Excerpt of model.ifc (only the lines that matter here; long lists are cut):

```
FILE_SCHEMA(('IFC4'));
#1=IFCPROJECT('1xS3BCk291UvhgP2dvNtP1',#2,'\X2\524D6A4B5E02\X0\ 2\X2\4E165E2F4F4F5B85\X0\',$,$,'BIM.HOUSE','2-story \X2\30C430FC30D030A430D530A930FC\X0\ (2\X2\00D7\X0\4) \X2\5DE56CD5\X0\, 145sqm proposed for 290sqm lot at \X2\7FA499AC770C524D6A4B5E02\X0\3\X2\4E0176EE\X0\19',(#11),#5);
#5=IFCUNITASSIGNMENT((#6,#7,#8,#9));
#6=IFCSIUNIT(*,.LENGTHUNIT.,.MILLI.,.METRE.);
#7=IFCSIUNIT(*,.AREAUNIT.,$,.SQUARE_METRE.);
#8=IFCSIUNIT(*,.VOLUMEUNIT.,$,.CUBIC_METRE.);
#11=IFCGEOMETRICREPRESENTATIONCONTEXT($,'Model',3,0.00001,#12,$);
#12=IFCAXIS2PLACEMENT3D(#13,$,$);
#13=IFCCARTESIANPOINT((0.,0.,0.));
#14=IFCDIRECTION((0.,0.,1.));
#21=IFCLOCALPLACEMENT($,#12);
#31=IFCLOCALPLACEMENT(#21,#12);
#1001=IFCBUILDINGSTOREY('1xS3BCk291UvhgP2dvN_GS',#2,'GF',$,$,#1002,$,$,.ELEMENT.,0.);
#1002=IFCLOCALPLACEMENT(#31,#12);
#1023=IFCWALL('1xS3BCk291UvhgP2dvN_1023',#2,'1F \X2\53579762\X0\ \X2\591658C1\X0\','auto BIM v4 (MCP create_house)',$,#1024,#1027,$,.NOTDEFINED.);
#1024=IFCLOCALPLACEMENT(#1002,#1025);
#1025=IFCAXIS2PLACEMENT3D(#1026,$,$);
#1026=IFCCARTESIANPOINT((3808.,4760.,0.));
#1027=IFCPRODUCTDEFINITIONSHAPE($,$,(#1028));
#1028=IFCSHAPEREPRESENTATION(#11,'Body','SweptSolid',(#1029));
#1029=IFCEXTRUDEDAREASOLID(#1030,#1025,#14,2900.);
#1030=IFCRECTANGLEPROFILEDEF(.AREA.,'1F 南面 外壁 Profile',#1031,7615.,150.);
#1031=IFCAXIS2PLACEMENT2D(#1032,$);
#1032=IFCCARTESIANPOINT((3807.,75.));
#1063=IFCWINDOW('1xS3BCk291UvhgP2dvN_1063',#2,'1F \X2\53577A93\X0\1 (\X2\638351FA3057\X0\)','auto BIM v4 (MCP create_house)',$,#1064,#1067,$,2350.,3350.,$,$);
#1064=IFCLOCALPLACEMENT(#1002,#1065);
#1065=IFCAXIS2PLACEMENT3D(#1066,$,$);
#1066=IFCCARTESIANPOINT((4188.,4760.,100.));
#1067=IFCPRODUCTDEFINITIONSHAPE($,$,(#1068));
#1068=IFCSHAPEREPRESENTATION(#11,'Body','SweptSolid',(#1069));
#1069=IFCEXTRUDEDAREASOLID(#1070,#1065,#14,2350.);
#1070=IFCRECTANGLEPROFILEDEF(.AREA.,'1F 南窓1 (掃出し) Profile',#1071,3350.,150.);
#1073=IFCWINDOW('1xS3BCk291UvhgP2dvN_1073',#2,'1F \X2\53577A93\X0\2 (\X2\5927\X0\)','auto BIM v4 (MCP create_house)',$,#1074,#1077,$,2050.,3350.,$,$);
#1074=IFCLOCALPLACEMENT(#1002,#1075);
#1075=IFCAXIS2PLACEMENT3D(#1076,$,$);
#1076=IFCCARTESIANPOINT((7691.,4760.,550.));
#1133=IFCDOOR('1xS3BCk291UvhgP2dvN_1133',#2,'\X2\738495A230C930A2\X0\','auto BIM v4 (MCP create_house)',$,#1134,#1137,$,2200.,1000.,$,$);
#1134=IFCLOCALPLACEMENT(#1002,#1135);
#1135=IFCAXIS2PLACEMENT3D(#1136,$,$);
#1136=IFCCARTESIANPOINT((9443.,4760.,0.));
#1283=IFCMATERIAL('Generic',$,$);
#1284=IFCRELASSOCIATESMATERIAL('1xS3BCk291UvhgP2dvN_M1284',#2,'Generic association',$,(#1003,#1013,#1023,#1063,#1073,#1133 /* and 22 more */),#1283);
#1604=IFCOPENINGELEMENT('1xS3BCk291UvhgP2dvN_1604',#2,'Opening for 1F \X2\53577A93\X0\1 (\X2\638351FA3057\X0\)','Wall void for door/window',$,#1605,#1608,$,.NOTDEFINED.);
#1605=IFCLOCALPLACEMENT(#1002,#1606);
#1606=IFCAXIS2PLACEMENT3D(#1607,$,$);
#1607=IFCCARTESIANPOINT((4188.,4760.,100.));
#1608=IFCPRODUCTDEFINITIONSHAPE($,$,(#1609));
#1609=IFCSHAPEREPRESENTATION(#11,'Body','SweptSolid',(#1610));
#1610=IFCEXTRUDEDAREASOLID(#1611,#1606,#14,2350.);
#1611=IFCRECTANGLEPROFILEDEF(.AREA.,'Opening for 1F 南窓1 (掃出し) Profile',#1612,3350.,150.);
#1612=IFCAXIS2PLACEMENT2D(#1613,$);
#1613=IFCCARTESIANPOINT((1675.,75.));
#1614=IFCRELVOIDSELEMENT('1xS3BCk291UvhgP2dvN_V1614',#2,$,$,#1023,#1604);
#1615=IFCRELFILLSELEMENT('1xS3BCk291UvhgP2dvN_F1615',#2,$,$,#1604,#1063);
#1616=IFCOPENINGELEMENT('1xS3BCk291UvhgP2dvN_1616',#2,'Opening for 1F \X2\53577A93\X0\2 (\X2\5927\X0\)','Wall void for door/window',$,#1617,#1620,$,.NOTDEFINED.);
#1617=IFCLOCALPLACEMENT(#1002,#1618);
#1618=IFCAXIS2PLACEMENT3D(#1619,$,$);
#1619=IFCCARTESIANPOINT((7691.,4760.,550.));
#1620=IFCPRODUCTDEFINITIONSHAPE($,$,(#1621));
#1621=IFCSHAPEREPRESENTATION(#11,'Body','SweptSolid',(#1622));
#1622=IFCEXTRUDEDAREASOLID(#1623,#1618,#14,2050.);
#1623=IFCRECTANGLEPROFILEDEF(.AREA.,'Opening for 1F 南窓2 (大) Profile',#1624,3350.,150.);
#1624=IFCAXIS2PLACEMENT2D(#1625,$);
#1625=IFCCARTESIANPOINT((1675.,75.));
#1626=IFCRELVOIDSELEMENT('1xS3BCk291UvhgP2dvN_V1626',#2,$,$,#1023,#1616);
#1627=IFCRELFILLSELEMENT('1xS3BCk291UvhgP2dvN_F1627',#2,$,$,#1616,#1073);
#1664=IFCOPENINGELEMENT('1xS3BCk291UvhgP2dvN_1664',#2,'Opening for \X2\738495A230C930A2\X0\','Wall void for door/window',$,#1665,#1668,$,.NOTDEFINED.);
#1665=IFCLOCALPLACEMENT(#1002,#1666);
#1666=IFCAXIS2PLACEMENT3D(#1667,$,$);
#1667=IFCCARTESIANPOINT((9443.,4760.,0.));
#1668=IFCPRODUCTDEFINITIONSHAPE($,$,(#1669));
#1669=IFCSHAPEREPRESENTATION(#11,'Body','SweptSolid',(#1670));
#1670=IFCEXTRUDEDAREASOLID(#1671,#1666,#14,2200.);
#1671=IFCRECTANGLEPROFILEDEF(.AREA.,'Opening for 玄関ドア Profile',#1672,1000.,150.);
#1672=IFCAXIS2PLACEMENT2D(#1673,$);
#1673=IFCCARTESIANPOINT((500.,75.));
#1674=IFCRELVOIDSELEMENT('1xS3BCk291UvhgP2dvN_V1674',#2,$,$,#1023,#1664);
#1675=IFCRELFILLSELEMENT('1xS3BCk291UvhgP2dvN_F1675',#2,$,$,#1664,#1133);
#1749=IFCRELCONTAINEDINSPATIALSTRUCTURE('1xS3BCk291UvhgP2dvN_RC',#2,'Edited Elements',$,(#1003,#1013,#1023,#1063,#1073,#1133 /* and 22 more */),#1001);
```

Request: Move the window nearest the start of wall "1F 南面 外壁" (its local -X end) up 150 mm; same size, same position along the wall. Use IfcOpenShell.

```python
import numpy as np
import ifcopenshell
import ifcopenshell.api.geometry
import ifcopenshell.util.placement
import ifcopenshell.util.unit

model = ifcopenshell.open("model.ifc")
unit_scale = ifcopenshell.util.unit.calculate_unit_scale(model)

window = model.by_id(1063)
opening = window.FillsVoids[0].RelatingOpeningElement
dz = 0.15 / unit_scale

shift = np.array([0.0, 0.0, dz])
# The window is not placed relative to its opening, so move both.
for product in (opening, window):
    matrix = ifcopenshell.util.placement.get_local_placement(product.ObjectPlacement)
    matrix[:3, 3] += shift
    ifcopenshell.api.geometry.edit_object_placement(model, product=product, matrix=matrix, is_si=False)

print(f"moved by {dz * unit_scale:+.3f} m")

model.write("model_updated.ifc")
```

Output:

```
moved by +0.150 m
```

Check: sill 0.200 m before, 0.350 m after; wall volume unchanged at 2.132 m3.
